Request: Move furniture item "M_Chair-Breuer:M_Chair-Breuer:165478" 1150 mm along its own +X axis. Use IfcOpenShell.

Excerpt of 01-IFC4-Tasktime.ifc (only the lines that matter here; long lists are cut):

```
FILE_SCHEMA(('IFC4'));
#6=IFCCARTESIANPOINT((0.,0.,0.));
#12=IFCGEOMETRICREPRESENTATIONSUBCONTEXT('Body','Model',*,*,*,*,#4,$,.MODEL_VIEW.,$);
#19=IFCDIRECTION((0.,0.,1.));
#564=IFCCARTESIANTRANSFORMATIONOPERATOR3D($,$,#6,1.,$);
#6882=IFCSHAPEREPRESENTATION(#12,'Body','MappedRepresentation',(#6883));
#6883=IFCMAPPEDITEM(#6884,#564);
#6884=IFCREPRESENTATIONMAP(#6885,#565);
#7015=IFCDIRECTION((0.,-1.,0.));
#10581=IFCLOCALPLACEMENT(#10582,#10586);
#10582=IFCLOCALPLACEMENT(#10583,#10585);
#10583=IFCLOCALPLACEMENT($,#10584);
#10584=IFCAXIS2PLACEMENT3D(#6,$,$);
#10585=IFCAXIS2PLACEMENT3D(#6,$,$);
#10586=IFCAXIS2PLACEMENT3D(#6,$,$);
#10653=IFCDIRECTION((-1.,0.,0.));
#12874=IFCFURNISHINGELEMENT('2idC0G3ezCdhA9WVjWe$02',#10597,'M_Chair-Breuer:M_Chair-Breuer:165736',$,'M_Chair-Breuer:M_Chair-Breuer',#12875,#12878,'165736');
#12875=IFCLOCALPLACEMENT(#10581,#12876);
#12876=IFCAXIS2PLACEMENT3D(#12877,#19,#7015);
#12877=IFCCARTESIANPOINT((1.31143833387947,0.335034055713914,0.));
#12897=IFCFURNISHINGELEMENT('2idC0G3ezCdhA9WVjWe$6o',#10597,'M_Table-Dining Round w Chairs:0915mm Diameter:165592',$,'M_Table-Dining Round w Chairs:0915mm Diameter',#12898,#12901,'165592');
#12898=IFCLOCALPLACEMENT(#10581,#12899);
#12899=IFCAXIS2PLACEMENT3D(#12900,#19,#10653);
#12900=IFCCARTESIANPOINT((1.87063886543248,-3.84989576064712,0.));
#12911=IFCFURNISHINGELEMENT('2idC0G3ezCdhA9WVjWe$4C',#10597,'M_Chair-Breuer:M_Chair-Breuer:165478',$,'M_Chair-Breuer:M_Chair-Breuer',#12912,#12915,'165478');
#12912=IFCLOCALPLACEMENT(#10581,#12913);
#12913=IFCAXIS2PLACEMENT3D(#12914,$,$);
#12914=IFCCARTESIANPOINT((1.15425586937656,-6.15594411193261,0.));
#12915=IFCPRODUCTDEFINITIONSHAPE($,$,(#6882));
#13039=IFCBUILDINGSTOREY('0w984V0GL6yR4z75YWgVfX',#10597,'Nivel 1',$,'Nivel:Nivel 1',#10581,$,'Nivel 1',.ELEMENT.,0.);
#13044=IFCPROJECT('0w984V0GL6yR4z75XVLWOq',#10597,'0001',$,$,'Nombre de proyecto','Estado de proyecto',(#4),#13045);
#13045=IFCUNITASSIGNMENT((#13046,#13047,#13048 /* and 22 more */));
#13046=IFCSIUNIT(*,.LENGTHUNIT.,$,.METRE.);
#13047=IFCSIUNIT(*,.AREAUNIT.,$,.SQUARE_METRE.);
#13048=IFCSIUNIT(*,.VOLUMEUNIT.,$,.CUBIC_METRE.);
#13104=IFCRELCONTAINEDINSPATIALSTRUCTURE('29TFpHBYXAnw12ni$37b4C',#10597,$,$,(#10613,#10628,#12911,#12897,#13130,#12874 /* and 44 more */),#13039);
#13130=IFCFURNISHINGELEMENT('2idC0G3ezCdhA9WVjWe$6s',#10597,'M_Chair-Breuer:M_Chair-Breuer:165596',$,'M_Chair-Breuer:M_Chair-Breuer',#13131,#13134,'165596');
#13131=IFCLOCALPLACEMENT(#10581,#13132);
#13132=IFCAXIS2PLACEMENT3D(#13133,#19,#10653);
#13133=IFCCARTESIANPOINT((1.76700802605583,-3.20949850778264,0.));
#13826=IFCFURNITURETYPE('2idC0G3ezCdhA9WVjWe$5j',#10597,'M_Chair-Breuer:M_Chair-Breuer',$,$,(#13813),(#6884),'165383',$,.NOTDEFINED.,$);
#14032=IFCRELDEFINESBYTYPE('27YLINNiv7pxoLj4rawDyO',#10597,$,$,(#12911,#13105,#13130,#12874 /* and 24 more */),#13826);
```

```python
import ifcopenshell
import ifcopenshell.api.geometry
import ifcopenshell.util.placement
import ifcopenshell.util.unit

model = ifcopenshell.open("01-IFC4-Tasktime.ifc")
unit_scale = ifcopenshell.util.unit.calculate_unit_scale(model)

item = model.by_guid("2idC0G3ezCdhA9WVjWe$4C")
matrix = ifcopenshell.util.placement.get_local_placement(item.ObjectPlacement)
matrix[:3, 3] += matrix[:3, 0] * 1.15 / unit_scale
ifcopenshell.api.geometry.edit_object_placement(model, product=item, matrix=matrix, is_si=False)

print(ifcopenshell.util.placement.get_local_placement(item.ObjectPlacement).round(3) + 0.0)

model.write("01-IFC4-Tasktime_updated.ifc")
```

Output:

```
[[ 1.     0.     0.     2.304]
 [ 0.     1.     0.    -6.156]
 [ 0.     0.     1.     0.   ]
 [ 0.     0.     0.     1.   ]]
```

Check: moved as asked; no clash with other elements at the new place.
